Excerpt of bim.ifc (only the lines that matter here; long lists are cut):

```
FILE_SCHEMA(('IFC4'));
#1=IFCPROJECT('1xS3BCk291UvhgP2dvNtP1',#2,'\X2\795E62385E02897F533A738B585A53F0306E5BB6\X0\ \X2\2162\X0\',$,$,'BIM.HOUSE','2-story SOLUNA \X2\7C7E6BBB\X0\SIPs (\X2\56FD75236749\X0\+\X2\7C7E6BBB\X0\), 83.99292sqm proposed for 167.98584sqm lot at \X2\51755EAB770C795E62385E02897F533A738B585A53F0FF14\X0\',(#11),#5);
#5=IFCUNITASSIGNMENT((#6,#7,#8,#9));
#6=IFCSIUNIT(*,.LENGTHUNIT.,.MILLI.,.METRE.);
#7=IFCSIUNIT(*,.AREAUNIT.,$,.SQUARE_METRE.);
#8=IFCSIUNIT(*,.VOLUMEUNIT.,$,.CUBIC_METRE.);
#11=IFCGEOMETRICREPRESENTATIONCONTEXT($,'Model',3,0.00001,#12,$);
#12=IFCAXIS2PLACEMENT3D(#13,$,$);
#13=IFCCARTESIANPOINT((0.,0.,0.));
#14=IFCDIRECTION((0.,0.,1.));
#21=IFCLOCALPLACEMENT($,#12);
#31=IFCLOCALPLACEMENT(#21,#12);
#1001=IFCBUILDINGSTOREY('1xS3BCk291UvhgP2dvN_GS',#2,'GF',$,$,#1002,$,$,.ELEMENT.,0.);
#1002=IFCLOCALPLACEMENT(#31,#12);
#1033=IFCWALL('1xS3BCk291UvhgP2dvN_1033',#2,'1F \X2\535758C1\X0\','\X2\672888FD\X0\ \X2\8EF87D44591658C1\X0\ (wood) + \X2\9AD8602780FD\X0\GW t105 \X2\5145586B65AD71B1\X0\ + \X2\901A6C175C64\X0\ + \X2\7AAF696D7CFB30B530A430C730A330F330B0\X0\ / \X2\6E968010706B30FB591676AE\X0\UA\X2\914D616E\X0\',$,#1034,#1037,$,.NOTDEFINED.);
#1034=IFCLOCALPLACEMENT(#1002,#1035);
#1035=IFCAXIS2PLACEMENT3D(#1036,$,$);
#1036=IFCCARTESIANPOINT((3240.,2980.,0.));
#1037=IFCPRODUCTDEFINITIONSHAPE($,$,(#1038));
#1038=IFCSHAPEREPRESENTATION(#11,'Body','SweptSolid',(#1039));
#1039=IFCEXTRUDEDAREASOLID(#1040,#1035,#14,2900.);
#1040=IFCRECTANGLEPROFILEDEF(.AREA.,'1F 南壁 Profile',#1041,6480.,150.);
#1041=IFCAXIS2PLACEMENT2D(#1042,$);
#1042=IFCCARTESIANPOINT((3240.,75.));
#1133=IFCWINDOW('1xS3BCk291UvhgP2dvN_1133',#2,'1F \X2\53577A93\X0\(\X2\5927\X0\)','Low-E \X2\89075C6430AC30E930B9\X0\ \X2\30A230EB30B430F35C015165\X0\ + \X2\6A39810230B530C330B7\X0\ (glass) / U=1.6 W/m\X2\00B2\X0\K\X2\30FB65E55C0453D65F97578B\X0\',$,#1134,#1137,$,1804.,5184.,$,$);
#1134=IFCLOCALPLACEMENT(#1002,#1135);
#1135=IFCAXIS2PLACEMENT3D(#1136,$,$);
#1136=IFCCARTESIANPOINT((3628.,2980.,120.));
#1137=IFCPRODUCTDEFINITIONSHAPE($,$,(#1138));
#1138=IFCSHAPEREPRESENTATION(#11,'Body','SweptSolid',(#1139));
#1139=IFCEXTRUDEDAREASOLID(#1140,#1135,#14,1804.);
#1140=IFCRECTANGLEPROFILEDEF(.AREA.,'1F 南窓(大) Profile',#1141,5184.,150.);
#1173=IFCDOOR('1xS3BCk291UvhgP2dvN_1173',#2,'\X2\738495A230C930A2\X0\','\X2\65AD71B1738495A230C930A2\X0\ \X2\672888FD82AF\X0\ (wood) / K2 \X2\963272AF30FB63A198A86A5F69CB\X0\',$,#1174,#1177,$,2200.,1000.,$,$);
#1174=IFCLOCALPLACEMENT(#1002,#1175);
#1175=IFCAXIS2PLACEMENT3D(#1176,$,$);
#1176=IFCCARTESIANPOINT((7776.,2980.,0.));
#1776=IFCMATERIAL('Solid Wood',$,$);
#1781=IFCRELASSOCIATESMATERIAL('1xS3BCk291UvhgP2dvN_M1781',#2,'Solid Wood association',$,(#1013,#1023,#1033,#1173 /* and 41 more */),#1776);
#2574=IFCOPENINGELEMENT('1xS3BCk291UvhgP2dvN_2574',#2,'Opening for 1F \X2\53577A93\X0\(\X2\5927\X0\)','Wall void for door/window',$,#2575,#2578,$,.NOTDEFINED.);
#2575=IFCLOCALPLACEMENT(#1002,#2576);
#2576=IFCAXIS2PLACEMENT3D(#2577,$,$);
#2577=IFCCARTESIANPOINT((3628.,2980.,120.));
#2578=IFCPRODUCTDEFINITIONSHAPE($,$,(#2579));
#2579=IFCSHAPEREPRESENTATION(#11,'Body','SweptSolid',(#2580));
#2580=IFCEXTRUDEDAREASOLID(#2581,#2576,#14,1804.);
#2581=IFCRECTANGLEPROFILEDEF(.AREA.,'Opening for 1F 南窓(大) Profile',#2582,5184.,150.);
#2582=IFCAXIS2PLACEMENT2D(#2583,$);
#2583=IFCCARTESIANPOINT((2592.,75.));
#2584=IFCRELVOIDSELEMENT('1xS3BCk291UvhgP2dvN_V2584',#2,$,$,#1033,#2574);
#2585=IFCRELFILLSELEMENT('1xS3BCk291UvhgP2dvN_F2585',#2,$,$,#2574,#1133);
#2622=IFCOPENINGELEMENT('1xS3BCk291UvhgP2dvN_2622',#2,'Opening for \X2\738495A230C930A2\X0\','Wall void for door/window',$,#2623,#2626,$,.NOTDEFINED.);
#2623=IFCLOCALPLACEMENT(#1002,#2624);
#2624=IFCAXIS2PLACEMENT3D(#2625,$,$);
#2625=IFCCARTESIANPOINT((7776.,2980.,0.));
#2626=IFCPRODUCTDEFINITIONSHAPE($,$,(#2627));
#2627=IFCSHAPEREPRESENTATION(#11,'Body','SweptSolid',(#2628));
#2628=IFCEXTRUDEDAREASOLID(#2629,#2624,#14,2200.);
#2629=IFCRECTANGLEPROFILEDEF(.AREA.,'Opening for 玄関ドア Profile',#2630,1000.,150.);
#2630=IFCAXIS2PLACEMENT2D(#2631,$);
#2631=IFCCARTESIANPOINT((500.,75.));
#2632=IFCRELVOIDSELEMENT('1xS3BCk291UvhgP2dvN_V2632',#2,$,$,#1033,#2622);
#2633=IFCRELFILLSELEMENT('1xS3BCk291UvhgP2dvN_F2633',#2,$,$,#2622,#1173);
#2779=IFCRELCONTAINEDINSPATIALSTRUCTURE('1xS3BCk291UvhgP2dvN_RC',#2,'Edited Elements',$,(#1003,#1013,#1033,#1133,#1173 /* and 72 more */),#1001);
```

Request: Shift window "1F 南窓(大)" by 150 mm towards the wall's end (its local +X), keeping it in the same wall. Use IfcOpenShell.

```python
import ifcopenshell
import ifcopenshell.api.geometry
import ifcopenshell.util.placement
import ifcopenshell.util.unit

model = ifcopenshell.open("bim.ifc")
unit_scale = ifcopenshell.util.unit.calculate_unit_scale(model)

window = model.by_guid("1xS3BCk291UvhgP2dvN_1133")
opening = window.FillsVoids[0].RelatingOpeningElement
wall = opening.VoidsElements[0].RelatingBuildingElement

wall_matrix = ifcopenshell.util.placement.get_local_placement(wall.ObjectPlacement)
shift = wall_matrix[:3, 0] * 0.15 / unit_scale
before = ifcopenshell.util.placement.get_local_placement(window.ObjectPlacement)[:3, 3].copy()

# The window is not placed relative to its opening, so move both.
for product in (opening, window):
    matrix = ifcopenshell.util.placement.get_local_placement(product.ObjectPlacement)
    matrix[:3, 3] += shift
    ifcopenshell.api.geometry.edit_object_placement(model, product=product, matrix=matrix, is_si=False)

after = ifcopenshell.util.placement.get_local_placement(window.ObjectPlacement)[:3, 3]
print("window moved by", (after - before).round(3) + 0.0)

model.write("bim_updated.ifc")
```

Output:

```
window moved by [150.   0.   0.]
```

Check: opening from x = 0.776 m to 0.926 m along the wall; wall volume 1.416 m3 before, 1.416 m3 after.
